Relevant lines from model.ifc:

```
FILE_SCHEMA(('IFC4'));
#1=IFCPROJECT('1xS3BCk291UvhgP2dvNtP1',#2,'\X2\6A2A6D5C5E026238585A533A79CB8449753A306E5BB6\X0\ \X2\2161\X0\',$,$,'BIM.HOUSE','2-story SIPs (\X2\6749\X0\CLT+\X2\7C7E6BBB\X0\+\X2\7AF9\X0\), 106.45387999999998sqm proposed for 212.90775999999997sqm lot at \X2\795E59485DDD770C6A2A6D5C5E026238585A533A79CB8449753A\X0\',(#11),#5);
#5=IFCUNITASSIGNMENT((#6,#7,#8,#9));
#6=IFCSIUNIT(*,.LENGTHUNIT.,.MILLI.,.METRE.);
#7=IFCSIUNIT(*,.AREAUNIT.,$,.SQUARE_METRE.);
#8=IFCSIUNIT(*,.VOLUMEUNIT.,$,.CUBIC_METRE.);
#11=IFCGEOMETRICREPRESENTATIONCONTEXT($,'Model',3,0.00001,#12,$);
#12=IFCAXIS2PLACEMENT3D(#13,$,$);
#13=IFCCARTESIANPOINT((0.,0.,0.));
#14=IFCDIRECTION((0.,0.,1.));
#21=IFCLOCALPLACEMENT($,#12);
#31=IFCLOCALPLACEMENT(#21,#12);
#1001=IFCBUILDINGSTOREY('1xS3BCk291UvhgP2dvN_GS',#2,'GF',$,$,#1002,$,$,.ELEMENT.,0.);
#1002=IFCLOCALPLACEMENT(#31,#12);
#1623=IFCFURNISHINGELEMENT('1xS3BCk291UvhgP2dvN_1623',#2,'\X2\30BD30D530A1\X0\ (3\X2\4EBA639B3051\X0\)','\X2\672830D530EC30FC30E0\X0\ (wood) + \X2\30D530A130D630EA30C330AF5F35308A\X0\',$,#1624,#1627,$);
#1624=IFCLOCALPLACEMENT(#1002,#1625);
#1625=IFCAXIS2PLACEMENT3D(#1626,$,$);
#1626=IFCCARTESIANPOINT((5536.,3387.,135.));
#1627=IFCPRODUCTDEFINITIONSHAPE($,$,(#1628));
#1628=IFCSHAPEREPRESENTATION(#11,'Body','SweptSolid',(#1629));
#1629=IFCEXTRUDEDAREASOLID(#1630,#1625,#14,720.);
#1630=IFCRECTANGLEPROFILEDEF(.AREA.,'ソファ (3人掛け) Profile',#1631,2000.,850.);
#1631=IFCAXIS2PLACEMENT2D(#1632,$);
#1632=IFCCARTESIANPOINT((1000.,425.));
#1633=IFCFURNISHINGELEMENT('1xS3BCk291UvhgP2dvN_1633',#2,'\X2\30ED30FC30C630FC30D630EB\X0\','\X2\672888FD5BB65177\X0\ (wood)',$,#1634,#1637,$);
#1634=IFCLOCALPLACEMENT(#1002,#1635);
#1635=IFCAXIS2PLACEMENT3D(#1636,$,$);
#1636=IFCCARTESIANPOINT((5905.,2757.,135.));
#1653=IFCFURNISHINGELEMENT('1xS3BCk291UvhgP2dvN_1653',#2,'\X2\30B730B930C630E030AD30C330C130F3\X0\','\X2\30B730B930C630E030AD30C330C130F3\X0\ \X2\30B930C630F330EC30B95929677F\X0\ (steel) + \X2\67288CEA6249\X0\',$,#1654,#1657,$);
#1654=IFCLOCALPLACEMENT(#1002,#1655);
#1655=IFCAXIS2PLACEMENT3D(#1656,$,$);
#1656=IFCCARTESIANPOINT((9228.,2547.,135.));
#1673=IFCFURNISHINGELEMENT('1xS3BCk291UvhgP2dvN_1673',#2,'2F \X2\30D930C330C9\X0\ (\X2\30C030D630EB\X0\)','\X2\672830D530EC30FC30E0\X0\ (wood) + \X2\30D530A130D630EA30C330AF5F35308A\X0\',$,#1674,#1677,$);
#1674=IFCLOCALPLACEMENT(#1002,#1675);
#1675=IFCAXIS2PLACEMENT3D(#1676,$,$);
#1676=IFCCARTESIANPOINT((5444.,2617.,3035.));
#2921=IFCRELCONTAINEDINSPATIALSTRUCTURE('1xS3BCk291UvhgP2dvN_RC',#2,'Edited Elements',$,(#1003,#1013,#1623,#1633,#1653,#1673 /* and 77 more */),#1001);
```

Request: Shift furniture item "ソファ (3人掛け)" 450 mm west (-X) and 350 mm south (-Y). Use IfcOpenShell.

```python
import ifcopenshell
import ifcopenshell.api.geometry
import ifcopenshell.util.placement
import ifcopenshell.util.unit

model = ifcopenshell.open("model.ifc")
unit_scale = ifcopenshell.util.unit.calculate_unit_scale(model)

item = model.by_guid("1xS3BCk291UvhgP2dvN_1623")
matrix = ifcopenshell.util.placement.get_local_placement(item.ObjectPlacement)
matrix[0, 3] -= 0.45 / unit_scale
matrix[1, 3] -= 0.35 / unit_scale
ifcopenshell.api.geometry.edit_object_placement(model, product=item, matrix=matrix, is_si=False)

print(ifcopenshell.util.placement.get_local_placement(item.ObjectPlacement).round(3) + 0.0)

model.write("model_rev.ifc")
```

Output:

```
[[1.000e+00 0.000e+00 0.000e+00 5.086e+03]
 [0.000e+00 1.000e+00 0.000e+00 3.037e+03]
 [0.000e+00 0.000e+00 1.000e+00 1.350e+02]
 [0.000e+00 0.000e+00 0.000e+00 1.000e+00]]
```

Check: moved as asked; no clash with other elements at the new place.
